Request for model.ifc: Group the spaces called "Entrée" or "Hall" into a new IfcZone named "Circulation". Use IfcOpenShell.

First a look at what the model holds.

```python
import ifcopenshell

model = ifcopenshell.open("model.ifc")
print(model.schema)
seen = {}
for space in model.by_type("IfcSpace"):
    seen[space.LongName] = seen.get(space.LongName, 0) + 1
for name, count in sorted(seen.items(), key=str):
    print(count, "x", name)
print("zones:", [z.Name for z in model.by_type("IfcZone")][:20])
```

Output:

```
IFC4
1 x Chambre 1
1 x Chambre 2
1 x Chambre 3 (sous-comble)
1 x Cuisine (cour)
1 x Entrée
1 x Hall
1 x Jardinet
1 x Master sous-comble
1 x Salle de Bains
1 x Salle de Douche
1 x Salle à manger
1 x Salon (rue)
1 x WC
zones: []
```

```python
import ifcopenshell
import ifcopenshell.api.group
import ifcopenshell.api.root

model = ifcopenshell.open("model.ifc")

names = {"Entrée", "Hall"}
spaces = [s for s in model.by_type("IfcSpace") if s.LongName in names]

zone = ifcopenshell.api.root.create_entity(model, ifc_class="IfcZone", name="Circulation")
ifcopenshell.api.group.assign_group(model, products=spaces, group=zone)
print(len(spaces), "spaces in", zone.Name)

model.write("model_rev.ifc")
```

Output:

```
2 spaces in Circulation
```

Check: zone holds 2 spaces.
